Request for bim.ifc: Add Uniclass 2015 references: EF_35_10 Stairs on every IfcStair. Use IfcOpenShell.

First a look at what the model holds.

```python
import ifcopenshell

model = ifcopenshell.open("bim.ifc")
print(model.schema)
print("classifications:", [c.Name for c in model.by_type("IfcClassification")])
for ifc_class in ("IfcDoor", "IfcRoof", "IfcStair", "IfcWall", "IfcWindow"):
    print(ifc_class, len(model.by_type(ifc_class)))
```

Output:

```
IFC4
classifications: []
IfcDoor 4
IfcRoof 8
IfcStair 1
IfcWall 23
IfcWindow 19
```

```python
import ifcopenshell
import ifcopenshell.api.classification

model = ifcopenshell.open("bim.ifc")

system = ifcopenshell.api.classification.add_classification(model, classification="Uniclass 2015")

codes = {
    "IfcStair": ("EF_35_10", "Stairs"),
}
for ifc_class, (code, name) in codes.items():
    products = model.by_type(ifc_class)
    ifcopenshell.api.classification.add_reference(
        model, products=products, classification=system, identification=code, name=name
    )
    print(code, len(products))

model.write("bim_rev.ifc")
```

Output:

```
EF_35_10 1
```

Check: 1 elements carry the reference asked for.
